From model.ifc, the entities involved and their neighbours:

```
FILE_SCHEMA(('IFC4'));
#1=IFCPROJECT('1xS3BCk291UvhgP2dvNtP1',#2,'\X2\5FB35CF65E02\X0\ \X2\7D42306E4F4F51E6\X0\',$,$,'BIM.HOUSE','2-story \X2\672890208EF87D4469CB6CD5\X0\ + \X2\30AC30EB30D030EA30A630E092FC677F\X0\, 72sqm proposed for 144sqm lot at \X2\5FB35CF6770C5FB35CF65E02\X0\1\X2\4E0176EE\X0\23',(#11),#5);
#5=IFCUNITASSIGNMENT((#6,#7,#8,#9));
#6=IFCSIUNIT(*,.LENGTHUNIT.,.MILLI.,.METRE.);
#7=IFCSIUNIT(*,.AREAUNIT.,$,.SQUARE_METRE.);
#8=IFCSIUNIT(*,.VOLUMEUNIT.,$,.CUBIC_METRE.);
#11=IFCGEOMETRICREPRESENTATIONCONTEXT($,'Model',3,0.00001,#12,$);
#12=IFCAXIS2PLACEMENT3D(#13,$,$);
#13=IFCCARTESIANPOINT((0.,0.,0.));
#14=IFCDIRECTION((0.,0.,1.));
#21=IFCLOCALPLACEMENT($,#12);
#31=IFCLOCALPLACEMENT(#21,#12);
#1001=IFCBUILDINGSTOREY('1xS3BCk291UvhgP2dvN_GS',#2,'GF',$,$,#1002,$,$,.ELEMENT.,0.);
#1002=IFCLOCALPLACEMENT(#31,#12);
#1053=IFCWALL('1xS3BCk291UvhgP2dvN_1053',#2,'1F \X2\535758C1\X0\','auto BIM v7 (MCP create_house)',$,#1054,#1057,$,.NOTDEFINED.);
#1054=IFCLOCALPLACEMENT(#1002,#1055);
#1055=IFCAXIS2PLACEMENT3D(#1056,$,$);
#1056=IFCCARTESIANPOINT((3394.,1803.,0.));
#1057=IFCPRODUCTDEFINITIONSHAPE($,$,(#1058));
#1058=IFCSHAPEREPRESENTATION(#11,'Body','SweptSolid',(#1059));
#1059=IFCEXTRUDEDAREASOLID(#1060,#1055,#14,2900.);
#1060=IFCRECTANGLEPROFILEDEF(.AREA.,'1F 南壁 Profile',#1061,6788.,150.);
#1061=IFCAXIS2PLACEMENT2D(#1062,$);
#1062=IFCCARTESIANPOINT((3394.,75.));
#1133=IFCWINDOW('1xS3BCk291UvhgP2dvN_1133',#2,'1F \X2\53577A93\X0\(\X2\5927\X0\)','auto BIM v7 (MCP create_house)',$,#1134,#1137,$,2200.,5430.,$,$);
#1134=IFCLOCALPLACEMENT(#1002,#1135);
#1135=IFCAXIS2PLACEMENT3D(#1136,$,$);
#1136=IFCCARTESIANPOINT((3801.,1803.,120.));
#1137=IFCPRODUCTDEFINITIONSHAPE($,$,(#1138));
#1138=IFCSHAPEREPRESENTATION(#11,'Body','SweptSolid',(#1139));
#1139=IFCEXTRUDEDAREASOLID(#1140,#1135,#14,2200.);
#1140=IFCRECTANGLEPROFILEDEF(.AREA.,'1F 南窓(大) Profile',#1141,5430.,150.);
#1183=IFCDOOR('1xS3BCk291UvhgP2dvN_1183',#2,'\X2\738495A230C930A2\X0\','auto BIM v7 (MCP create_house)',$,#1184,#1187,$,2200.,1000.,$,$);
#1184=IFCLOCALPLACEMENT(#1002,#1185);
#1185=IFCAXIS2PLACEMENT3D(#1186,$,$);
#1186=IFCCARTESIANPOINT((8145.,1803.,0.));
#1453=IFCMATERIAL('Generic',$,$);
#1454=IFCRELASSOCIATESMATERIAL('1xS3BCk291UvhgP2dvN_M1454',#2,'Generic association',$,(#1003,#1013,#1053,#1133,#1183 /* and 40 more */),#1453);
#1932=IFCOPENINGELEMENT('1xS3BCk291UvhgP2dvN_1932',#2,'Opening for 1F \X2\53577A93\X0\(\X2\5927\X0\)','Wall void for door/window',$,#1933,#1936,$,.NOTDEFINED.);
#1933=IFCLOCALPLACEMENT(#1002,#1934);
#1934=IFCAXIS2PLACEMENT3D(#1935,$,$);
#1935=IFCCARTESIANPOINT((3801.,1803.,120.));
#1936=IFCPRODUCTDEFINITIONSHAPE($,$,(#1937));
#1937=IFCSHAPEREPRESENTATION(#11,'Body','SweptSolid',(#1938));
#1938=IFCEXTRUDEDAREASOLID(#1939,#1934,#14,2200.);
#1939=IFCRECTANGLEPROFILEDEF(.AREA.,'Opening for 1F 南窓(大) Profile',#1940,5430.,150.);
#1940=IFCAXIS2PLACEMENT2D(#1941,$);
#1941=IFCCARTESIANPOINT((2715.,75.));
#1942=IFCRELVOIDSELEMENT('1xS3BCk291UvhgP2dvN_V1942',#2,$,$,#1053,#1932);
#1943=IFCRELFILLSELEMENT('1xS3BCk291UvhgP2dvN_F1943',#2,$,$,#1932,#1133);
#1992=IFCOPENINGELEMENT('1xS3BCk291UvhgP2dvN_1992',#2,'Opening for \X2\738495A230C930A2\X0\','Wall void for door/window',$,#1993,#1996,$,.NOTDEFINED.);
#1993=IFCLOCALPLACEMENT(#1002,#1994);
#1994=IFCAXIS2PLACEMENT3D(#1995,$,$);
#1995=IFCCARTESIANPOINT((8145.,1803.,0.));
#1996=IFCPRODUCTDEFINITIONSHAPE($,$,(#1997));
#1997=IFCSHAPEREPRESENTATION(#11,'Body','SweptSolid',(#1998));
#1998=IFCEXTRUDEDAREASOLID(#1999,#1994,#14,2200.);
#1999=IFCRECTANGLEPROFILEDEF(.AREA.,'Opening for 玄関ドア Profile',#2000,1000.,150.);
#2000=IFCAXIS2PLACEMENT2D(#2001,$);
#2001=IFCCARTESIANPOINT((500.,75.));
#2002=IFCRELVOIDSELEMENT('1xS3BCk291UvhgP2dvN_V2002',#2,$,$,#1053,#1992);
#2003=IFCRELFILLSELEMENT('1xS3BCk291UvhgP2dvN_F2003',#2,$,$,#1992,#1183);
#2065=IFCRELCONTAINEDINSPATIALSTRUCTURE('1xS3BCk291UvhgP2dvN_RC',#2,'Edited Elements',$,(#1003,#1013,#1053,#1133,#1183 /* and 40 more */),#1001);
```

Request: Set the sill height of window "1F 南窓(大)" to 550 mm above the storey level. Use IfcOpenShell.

```python
import numpy as np
import ifcopenshell
import ifcopenshell.api.geometry
import ifcopenshell.geom
import ifcopenshell.util.element
import ifcopenshell.util.placement
import ifcopenshell.util.shape
import ifcopenshell.util.unit

model = ifcopenshell.open("model.ifc")
unit_scale = ifcopenshell.util.unit.calculate_unit_scale(model)

window = model.by_guid("1xS3BCk291UvhgP2dvN_1133")
opening = window.FillsVoids[0].RelatingOpeningElement
storey = ifcopenshell.util.element.get_container(window, ifc_class="IfcBuildingStorey")
level = ifcopenshell.util.placement.get_local_placement(storey.ObjectPlacement)[2, 3]

# The opening's origin need not be at the sill, so measure its lowest point.
shape = ifcopenshell.geom.create_shape(ifcopenshell.geom.settings(), opening)
bottom = ifcopenshell.util.shape.get_shape_bottom_elevation(shape, shape.geometry) / unit_scale
dz = level + 550.0 - bottom

shift = np.array([0.0, 0.0, dz])
# The window is not placed relative to its opening, so move both.
for product in (opening, window):
    matrix = ifcopenshell.util.placement.get_local_placement(product.ObjectPlacement)
    matrix[:3, 3] += shift
    ifcopenshell.api.geometry.edit_object_placement(model, product=product, matrix=matrix, is_si=False)

print(f"moved by {dz * unit_scale:+.3f} m")

model.write("model_updated.ifc")
```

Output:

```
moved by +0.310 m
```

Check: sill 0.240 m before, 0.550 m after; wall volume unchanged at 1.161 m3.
